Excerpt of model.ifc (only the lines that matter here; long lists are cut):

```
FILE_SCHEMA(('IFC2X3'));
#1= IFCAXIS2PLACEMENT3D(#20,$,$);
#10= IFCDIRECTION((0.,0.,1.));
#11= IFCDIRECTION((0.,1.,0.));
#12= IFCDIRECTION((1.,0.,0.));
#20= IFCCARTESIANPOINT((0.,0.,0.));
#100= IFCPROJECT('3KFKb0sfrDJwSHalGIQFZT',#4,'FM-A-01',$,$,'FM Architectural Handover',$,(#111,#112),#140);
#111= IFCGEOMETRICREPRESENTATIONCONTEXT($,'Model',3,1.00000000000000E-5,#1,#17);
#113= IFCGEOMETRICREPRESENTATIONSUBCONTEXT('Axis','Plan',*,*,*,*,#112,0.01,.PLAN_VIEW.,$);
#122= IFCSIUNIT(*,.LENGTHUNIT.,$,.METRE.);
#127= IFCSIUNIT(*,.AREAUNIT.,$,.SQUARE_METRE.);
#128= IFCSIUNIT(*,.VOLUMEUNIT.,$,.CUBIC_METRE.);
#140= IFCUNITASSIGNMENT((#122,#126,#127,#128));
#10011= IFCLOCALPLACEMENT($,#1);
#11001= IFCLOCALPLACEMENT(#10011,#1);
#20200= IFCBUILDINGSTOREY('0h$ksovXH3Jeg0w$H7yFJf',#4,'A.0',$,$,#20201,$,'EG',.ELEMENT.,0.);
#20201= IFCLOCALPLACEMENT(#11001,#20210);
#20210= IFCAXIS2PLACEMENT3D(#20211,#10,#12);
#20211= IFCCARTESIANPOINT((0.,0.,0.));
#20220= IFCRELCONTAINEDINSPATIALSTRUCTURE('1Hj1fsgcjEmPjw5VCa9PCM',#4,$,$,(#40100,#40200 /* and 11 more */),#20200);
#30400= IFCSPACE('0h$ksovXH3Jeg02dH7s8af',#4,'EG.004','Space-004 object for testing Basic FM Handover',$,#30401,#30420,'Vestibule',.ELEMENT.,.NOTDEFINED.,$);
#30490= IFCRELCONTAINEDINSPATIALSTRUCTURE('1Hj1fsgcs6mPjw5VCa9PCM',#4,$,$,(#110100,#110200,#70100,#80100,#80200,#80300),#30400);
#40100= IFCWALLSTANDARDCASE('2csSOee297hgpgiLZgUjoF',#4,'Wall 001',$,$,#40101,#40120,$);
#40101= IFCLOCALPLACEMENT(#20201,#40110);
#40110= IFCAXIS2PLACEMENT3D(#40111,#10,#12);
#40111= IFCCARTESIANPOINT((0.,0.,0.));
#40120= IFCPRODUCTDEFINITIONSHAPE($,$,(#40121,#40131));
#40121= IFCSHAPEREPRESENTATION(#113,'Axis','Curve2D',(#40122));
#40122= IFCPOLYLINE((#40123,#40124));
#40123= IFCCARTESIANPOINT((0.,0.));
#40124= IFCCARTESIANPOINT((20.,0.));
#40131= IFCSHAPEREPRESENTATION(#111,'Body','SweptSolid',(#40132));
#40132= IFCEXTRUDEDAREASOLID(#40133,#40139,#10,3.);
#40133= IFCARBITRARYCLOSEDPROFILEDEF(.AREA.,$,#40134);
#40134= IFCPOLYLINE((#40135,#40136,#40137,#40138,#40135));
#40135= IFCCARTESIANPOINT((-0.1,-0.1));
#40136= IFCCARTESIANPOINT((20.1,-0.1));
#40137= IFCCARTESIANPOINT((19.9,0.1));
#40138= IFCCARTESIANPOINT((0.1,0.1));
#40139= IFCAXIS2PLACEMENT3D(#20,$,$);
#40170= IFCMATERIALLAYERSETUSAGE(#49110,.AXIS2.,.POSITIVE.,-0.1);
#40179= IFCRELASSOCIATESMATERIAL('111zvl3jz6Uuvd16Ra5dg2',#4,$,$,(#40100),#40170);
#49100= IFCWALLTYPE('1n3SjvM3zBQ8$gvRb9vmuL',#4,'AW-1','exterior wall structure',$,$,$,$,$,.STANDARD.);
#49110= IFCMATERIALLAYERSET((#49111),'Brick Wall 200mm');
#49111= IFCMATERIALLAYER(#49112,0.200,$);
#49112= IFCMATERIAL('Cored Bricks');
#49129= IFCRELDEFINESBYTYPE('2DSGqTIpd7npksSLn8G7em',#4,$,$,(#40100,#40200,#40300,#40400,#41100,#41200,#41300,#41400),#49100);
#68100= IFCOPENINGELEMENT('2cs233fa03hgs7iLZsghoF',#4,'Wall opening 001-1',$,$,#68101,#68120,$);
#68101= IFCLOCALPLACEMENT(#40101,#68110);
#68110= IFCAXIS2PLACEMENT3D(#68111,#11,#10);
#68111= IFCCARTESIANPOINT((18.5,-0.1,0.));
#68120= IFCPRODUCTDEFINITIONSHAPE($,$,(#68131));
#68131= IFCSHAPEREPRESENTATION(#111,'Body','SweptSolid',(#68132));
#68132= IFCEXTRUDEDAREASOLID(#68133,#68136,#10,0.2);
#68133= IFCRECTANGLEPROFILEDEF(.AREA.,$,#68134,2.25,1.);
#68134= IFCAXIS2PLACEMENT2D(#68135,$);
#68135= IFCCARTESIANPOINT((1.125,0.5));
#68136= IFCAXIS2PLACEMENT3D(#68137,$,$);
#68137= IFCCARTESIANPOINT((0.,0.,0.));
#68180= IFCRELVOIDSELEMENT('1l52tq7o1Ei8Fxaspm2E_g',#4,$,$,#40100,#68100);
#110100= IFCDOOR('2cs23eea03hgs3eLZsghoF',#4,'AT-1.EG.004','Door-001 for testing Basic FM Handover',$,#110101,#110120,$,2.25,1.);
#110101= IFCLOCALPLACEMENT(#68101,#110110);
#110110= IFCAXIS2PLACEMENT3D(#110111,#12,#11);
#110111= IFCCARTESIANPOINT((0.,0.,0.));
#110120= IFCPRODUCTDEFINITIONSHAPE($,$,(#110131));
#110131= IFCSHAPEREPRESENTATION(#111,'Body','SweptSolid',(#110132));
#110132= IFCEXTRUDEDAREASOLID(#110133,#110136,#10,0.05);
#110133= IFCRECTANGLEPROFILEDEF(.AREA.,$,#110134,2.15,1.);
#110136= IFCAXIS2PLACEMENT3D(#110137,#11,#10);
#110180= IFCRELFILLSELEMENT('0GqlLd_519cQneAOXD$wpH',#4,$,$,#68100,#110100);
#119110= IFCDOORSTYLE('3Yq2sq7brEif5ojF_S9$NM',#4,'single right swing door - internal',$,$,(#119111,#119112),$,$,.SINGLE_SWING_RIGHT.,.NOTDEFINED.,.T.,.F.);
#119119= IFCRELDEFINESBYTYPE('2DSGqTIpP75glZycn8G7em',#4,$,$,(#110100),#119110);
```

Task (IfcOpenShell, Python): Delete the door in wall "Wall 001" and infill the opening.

```python
import ifcopenshell
import ifcopenshell.api.feature
import ifcopenshell.api.root
import ifcopenshell.geom
import ifcopenshell.util.shape

model = ifcopenshell.open("model.ifc")
settings = ifcopenshell.geom.settings()


def volume(element):
    """Net volume in cubic metres, openings subtracted."""
    shape = ifcopenshell.geom.create_shape(settings, element)
    return ifcopenshell.util.shape.get_volume(shape.geometry)


door = model.by_guid("2cs23eea03hgs3eLZsghoF")
opening = door.FillsVoids[0].RelatingOpeningElement
wall = opening.VoidsElements[0].RelatingBuildingElement
before = volume(wall)

ifcopenshell.api.root.remove_product(model, product=door)
ifcopenshell.api.feature.remove_feature(model, feature=opening)

after = volume(wall)

print(f"wall volume {before:.3f} -> {after:.3f} m3")

model.write("model-out.ifc")
```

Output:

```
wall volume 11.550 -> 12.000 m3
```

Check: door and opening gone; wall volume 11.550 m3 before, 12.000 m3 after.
